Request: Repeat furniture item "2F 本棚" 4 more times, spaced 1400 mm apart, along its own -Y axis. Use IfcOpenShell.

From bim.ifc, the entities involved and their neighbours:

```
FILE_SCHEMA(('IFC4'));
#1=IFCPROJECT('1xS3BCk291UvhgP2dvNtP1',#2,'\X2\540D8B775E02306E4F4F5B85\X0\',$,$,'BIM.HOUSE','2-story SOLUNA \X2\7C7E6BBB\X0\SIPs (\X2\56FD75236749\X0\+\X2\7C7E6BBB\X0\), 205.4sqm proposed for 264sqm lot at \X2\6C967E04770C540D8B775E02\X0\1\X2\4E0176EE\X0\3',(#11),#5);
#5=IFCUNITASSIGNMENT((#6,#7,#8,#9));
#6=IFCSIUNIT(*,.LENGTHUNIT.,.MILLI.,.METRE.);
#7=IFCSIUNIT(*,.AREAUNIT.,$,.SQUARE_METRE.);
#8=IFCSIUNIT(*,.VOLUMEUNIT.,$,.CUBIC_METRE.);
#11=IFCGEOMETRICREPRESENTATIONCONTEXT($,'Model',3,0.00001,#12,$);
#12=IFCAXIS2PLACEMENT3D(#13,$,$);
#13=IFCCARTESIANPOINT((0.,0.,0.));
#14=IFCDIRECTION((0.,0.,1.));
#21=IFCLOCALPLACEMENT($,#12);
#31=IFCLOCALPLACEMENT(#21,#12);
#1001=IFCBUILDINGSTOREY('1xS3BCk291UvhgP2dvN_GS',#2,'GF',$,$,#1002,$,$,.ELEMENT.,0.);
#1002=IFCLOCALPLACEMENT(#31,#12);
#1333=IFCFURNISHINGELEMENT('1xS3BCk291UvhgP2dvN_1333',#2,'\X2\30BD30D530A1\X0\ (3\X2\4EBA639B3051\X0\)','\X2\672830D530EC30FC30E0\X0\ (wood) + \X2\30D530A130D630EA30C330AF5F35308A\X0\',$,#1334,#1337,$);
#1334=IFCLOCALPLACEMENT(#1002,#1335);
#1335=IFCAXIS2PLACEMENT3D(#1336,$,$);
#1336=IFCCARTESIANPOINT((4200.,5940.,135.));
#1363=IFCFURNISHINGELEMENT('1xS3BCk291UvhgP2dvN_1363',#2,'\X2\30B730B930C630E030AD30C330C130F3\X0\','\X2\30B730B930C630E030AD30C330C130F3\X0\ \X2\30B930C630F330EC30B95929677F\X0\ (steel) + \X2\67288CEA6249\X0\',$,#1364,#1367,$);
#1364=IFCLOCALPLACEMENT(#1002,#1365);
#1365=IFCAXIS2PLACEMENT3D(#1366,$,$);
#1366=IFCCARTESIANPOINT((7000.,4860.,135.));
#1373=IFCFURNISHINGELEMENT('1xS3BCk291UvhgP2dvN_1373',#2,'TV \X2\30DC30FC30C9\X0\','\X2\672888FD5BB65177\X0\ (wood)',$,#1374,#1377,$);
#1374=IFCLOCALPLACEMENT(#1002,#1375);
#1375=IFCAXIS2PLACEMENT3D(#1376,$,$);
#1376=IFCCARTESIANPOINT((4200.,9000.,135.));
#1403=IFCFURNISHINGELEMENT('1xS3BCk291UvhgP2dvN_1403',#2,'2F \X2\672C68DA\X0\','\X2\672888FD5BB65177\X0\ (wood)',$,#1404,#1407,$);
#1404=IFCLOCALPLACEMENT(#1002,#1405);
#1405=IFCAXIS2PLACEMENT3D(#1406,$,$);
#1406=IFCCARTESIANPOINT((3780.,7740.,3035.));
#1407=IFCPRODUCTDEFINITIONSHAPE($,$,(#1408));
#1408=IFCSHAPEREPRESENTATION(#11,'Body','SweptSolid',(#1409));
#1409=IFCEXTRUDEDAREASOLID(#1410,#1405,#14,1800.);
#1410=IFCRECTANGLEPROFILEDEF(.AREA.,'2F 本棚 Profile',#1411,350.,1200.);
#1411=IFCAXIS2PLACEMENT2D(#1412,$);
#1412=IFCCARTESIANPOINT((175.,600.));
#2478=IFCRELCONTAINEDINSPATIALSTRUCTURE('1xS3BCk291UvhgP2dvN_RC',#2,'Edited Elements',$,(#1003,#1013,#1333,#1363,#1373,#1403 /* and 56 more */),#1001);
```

```python
import ifcopenshell
import ifcopenshell.api.geometry
import ifcopenshell.api.root
import ifcopenshell.util.element
import ifcopenshell.util.placement
import ifcopenshell.util.unit

model = ifcopenshell.open("bim.ifc")
unit_scale = ifcopenshell.util.unit.calculate_unit_scale(model)


def reuse_history(source, copy):
    """copy_class also copies each property set's owner history, people and application; keep the originals."""
    for rel in copy.IsDefinedBy:
        if rel.is_a("IfcRelDefinesByProperties") and (history := rel.RelatingPropertyDefinition.OwnerHistory):
            rel.RelatingPropertyDefinition.OwnerHistory = source.OwnerHistory
            ifcopenshell.util.element.remove_deep2(model, history)


source = model.by_guid("1xS3BCk291UvhgP2dvN_1403")
base = ifcopenshell.util.placement.get_local_placement(source.ObjectPlacement)
step = -base[:3, 1] * 1.4 / unit_scale

for i in range(1, 5):
    copy = ifcopenshell.api.root.copy_class(model, product=source)
    copy.Representation = ifcopenshell.util.element.copy_deep(
        model, source.Representation, exclude=["IfcGeometricRepresentationContext", "IfcRepresentationMap"]
    )
    reuse_history(source, copy)
    matrix = base.copy()
    matrix[:3, 3] += i * step
    print("added at", matrix[:3, 3].round(3) + 0.0)
    ifcopenshell.api.geometry.edit_object_placement(model, product=copy, matrix=matrix, is_si=False)

model.write("bim_rev.ifc")
```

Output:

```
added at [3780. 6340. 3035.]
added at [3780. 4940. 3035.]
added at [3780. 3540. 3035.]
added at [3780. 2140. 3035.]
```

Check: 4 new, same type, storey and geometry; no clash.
